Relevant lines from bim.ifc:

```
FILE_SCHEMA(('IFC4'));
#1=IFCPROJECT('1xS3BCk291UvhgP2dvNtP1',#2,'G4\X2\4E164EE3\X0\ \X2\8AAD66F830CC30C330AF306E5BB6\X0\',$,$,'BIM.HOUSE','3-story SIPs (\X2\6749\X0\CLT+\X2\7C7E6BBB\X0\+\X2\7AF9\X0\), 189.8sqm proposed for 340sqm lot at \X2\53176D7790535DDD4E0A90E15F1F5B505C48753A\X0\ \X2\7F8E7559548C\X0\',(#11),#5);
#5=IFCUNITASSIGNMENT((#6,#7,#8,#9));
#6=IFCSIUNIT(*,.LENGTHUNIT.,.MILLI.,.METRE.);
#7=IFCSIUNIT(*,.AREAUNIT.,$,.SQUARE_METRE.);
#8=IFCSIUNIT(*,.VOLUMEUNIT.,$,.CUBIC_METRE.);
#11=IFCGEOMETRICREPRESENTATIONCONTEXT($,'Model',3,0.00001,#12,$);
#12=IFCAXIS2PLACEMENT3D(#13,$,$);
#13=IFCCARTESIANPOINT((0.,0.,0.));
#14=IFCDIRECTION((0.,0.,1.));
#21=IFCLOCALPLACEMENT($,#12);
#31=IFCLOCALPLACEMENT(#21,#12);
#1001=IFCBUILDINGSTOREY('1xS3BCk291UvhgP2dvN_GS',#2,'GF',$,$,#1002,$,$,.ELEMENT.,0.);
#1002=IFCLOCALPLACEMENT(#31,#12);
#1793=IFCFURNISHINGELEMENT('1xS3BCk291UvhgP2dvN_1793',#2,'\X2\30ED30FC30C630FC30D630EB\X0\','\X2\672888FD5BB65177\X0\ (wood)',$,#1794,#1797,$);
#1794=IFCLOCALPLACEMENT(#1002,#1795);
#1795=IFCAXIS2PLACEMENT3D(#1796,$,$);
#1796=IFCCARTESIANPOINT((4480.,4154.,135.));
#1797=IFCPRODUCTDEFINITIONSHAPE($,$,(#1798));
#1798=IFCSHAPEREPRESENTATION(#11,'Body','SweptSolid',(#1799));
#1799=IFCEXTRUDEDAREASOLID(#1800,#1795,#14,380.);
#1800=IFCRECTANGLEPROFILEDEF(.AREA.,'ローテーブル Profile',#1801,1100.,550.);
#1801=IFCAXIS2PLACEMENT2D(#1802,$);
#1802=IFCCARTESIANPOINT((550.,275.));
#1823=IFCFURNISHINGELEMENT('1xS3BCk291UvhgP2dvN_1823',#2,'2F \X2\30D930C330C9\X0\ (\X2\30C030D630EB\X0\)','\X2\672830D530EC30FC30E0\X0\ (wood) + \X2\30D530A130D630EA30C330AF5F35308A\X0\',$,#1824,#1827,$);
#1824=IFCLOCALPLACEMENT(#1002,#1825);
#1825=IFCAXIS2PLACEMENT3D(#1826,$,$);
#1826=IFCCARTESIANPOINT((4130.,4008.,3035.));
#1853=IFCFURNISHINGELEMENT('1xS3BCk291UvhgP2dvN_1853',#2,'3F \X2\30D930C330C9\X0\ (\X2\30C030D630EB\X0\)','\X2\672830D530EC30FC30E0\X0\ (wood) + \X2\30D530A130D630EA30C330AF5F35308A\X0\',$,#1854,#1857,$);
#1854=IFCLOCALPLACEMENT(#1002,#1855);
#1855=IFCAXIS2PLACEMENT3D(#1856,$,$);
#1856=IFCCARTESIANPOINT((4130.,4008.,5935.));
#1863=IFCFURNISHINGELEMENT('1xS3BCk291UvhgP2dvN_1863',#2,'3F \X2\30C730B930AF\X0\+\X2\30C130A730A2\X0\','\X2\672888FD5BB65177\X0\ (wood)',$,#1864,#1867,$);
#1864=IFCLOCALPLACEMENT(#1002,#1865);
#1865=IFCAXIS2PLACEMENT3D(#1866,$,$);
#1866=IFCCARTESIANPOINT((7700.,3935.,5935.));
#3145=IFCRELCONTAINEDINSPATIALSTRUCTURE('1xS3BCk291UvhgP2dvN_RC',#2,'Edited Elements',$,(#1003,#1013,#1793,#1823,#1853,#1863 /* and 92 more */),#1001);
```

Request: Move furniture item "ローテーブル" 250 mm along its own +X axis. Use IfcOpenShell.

```python
import ifcopenshell
import ifcopenshell.api.geometry
import ifcopenshell.util.placement
import ifcopenshell.util.unit

model = ifcopenshell.open("bim.ifc")
unit_scale = ifcopenshell.util.unit.calculate_unit_scale(model)

item = model.by_guid("1xS3BCk291UvhgP2dvN_1793")
matrix = ifcopenshell.util.placement.get_local_placement(item.ObjectPlacement)
matrix[:3, 3] += matrix[:3, 0] * 0.25 / unit_scale
ifcopenshell.api.geometry.edit_object_placement(model, product=item, matrix=matrix, is_si=False)

print(ifcopenshell.util.placement.get_local_placement(item.ObjectPlacement).round(3) + 0.0)

model.write("bim_rev.ifc")
```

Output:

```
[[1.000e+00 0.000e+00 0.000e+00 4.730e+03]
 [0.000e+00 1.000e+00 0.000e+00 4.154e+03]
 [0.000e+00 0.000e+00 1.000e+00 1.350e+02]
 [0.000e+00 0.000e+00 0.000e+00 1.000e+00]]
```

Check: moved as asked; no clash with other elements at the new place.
